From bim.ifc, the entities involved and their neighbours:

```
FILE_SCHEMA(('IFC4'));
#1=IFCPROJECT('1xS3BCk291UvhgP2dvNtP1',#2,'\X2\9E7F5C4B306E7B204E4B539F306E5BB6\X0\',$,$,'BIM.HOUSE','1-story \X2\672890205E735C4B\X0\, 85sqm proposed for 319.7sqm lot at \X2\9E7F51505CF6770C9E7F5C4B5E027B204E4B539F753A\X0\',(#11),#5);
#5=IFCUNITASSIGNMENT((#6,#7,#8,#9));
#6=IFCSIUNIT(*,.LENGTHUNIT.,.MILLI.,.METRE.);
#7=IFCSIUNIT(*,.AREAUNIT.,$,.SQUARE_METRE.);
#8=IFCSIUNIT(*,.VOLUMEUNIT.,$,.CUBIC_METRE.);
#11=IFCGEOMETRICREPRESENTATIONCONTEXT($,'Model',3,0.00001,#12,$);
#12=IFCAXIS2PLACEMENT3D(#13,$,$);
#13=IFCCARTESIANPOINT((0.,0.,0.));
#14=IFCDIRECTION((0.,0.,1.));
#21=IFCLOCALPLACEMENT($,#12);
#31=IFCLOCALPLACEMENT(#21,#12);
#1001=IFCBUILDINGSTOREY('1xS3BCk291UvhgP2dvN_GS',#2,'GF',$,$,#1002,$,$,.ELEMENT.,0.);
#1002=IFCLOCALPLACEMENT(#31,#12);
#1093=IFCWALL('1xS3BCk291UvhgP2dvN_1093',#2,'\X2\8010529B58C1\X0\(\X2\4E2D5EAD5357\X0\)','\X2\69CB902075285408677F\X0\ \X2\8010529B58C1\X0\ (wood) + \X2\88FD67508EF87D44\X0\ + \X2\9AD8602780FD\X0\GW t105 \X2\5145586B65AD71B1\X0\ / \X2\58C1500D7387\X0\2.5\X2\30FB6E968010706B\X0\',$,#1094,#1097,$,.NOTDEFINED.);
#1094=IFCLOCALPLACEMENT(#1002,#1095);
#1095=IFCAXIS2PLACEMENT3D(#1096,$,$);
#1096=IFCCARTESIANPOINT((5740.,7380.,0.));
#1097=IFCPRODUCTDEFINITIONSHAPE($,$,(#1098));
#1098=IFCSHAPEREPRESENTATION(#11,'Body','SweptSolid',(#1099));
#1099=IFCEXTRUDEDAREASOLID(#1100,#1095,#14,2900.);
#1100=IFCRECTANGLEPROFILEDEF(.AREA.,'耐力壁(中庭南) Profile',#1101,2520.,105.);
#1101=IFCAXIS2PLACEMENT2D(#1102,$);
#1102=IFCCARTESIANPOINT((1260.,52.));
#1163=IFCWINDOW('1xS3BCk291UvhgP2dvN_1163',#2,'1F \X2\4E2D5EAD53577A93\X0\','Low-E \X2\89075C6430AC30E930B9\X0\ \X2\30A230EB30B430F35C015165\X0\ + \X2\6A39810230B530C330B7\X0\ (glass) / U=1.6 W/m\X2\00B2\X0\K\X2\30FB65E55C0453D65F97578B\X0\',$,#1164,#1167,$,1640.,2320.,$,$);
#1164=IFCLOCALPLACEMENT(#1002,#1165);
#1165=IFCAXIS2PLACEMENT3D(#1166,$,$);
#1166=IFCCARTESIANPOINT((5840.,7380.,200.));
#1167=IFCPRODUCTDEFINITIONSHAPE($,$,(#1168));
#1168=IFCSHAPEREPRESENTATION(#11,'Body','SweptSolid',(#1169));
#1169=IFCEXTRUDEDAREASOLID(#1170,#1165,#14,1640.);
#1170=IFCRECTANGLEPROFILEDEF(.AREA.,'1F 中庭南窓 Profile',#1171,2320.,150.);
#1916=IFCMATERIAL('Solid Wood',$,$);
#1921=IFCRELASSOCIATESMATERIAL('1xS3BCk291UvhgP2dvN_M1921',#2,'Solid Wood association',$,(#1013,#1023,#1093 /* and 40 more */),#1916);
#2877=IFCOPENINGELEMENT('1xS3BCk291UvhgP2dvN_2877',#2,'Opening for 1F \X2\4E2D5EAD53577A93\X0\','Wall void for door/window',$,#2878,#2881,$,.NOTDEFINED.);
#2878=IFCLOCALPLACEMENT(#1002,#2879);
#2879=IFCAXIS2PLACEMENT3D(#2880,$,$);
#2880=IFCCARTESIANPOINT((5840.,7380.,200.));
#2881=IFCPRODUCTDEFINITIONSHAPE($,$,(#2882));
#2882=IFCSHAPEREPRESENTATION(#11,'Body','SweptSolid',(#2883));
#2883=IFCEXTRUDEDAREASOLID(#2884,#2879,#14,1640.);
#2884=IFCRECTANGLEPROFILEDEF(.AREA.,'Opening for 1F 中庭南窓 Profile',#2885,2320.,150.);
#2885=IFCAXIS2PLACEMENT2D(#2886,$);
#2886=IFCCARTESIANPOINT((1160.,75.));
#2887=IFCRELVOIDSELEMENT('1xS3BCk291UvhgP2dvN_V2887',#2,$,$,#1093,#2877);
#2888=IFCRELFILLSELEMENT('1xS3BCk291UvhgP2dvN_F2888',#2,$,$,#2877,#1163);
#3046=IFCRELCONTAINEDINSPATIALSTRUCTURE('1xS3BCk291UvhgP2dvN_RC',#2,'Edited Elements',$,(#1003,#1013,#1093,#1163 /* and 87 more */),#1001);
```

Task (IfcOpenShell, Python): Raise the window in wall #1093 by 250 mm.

```python
import numpy as np
import ifcopenshell
import ifcopenshell.api.geometry
import ifcopenshell.util.placement
import ifcopenshell.util.unit

model = ifcopenshell.open("bim.ifc")
unit_scale = ifcopenshell.util.unit.calculate_unit_scale(model)

window = model.by_guid("1xS3BCk291UvhgP2dvN_1163")
opening = window.FillsVoids[0].RelatingOpeningElement
dz = 0.25 / unit_scale

shift = np.array([0.0, 0.0, dz])
# The window is not placed relative to its opening, so move both.
for product in (opening, window):
    matrix = ifcopenshell.util.placement.get_local_placement(product.ObjectPlacement)
    matrix[:3, 3] += shift
    ifcopenshell.api.geometry.edit_object_placement(model, product=product, matrix=matrix, is_si=False)

print(f"moved by {dz * unit_scale:+.3f} m")

model.write("bim_v2.ifc")
```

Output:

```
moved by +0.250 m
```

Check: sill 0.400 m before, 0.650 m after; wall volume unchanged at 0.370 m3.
